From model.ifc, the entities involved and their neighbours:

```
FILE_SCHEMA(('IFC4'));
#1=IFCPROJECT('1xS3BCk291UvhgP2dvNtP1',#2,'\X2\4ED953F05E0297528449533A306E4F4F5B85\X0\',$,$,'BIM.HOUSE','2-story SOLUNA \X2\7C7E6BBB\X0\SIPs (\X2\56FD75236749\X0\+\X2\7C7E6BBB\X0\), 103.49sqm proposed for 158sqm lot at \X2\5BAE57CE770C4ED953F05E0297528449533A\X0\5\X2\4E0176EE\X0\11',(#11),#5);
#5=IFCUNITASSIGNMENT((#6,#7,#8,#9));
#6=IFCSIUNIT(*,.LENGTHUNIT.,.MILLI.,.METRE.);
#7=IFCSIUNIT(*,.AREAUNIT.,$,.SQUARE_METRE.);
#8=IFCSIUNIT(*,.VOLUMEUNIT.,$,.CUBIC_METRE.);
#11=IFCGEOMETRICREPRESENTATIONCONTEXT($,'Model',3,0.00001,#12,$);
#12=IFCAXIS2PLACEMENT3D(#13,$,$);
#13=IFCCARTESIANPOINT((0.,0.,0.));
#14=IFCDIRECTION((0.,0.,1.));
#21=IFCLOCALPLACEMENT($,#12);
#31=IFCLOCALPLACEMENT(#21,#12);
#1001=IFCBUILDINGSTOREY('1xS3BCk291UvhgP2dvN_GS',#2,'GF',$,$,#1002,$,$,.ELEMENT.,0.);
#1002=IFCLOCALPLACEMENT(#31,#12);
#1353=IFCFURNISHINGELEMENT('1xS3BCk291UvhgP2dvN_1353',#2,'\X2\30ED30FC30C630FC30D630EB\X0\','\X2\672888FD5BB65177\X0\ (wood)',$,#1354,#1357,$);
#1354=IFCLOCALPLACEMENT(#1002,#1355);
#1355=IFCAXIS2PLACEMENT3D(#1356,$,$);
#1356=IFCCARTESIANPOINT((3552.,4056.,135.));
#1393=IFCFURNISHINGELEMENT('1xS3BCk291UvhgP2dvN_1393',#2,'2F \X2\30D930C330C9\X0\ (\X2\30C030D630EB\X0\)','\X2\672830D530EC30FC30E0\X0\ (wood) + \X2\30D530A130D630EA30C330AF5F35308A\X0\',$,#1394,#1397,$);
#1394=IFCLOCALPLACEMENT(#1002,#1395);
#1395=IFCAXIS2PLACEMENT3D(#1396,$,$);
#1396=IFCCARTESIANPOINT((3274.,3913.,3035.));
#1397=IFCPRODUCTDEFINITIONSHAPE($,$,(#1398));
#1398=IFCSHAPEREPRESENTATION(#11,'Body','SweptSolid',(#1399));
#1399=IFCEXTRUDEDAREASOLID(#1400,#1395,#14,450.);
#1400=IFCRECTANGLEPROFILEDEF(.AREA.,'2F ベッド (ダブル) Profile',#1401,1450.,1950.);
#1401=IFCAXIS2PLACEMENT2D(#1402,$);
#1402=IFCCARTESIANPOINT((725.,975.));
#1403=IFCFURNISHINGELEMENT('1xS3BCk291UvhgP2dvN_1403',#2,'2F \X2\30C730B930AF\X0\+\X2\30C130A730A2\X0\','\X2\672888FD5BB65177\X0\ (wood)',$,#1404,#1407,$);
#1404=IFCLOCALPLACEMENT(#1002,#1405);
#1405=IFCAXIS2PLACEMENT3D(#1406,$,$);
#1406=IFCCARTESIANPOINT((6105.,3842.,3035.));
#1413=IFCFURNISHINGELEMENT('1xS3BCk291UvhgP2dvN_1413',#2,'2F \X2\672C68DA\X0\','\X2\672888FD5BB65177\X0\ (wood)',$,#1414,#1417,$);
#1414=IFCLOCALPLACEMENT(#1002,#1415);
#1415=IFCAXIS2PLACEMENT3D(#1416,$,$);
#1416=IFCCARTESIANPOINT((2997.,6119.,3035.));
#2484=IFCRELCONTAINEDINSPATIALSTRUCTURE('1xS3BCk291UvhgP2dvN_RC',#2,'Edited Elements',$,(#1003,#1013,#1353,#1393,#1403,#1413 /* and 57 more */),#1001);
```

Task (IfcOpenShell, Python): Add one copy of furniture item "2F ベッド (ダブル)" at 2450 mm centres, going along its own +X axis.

```python
import ifcopenshell
import ifcopenshell.api.geometry
import ifcopenshell.api.root
import ifcopenshell.util.element
import ifcopenshell.util.placement
import ifcopenshell.util.unit

model = ifcopenshell.open("model.ifc")
unit_scale = ifcopenshell.util.unit.calculate_unit_scale(model)


def reuse_history(source, copy):
    """copy_class also copies each property set's owner history, people and application; keep the originals."""
    for rel in copy.IsDefinedBy:
        if rel.is_a("IfcRelDefinesByProperties") and (history := rel.RelatingPropertyDefinition.OwnerHistory):
            rel.RelatingPropertyDefinition.OwnerHistory = source.OwnerHistory
            ifcopenshell.util.element.remove_deep2(model, history)


source = model.by_guid("1xS3BCk291UvhgP2dvN_1393")
base = ifcopenshell.util.placement.get_local_placement(source.ObjectPlacement)
step = base[:3, 0] * 2.45 / unit_scale

for i in range(1, 2):
    copy = ifcopenshell.api.root.copy_class(model, product=source)
    copy.Representation = ifcopenshell.util.element.copy_deep(
        model, source.Representation, exclude=["IfcGeometricRepresentationContext", "IfcRepresentationMap"]
    )
    reuse_history(source, copy)
    matrix = base.copy()
    matrix[:3, 3] += i * step
    print("added at", matrix[:3, 3].round(3) + 0.0)
    ifcopenshell.api.geometry.edit_object_placement(model, product=copy, matrix=matrix, is_si=False)

model.write("model-out.ifc")
```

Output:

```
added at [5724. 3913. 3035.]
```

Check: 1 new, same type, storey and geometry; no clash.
